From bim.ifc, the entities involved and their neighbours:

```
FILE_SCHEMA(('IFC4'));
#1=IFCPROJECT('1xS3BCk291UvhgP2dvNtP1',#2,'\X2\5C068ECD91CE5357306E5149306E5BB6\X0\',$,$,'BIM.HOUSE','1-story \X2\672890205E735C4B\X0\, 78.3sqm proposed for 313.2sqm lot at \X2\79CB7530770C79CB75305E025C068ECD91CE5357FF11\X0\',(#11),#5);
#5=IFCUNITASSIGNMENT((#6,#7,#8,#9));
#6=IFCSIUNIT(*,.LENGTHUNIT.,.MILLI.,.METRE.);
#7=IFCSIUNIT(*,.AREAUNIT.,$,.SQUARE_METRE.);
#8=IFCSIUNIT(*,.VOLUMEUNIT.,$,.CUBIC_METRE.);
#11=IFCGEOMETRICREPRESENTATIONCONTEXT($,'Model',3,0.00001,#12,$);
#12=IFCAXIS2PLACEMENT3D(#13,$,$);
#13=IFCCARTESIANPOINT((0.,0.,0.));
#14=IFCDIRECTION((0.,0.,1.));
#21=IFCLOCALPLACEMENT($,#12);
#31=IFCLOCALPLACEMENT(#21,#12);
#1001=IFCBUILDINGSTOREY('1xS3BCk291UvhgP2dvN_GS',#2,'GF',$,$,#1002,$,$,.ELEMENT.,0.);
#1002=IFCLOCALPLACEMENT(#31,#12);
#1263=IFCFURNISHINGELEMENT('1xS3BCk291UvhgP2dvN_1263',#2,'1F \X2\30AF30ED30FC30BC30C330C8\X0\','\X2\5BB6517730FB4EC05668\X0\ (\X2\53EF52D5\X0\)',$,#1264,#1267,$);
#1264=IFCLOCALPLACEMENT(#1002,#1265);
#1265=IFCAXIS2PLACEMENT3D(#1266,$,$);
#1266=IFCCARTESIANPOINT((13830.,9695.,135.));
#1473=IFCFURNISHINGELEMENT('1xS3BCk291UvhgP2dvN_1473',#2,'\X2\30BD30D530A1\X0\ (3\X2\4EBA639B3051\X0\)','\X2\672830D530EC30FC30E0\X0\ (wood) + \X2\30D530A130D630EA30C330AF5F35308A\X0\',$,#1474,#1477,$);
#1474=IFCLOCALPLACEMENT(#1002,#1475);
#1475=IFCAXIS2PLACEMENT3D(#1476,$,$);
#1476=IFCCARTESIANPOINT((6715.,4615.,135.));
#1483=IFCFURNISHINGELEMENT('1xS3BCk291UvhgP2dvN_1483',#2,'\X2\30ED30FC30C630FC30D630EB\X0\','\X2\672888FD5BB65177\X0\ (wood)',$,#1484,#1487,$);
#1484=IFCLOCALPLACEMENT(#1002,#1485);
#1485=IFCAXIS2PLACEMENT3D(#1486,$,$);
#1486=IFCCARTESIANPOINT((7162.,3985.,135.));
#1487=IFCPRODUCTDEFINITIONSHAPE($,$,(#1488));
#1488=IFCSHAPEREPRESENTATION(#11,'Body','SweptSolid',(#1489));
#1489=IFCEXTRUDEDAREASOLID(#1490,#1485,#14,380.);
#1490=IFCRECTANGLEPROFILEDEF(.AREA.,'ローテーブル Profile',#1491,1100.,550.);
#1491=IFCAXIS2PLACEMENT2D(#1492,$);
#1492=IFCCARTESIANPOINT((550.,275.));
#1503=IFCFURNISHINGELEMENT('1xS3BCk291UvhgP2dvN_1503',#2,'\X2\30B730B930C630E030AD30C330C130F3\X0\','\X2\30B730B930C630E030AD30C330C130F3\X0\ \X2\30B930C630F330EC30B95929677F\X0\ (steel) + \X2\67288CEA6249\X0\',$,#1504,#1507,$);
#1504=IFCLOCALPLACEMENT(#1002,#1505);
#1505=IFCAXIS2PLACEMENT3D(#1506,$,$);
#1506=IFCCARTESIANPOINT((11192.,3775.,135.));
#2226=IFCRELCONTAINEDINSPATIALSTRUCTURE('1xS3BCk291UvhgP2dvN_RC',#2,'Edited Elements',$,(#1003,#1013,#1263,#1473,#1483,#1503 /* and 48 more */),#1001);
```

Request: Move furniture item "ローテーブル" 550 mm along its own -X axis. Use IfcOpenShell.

```python
import ifcopenshell
import ifcopenshell.api.geometry
import ifcopenshell.util.placement

model = ifcopenshell.open("bim.ifc")

item = model.by_guid("1xS3BCk291UvhgP2dvN_1483")
matrix = ifcopenshell.util.placement.get_local_placement(item.ObjectPlacement)
matrix[:3, 3] -= matrix[:3, 0] * 550.0
ifcopenshell.api.geometry.edit_object_placement(model, product=item, matrix=matrix, is_si=False)

print(ifcopenshell.util.placement.get_local_placement(item.ObjectPlacement).round(3) + 0.0)

model.write("bim_updated.ifc")
```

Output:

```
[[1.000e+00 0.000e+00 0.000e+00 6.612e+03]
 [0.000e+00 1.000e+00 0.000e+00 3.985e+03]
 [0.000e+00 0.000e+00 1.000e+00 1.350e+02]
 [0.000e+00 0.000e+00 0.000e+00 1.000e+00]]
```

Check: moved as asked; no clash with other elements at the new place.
